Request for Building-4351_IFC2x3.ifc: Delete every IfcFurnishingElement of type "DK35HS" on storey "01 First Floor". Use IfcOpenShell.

First a look at what the model holds.

```python
import ifcopenshell
import ifcopenshell.util.element

model = ifcopenshell.open("Building-4351_IFC2x3.ifc")
print(model.schema)
storey = next(s for s in model.by_type("IfcBuildingStorey") if s.Name == "01 First Floor")
furniture = [e for e in ifcopenshell.util.element.get_decomposition(storey) if e.is_a("IfcFurnishingElement")]
seen = {}
for e in furniture:
    element_type = ifcopenshell.util.element.get_type(e)
    name = element_type.Name if element_type not in (None, e) else None
    seen[name] = seen.get(name, 0) + 1
for name, count in sorted(seen.items(), key=str):
    print(count, "x", name)
```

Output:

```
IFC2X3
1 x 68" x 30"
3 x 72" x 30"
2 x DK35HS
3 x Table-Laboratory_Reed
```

```python
import ifcopenshell
import ifcopenshell.api.root
import ifcopenshell.util.element

model = ifcopenshell.open("Building-4351_IFC2x3.ifc")

storey = next(s for s in model.by_type("IfcBuildingStorey") if s.Name == "01 First Floor")
furniture = [e for e in ifcopenshell.util.element.get_decomposition(storey) if e.is_a("IfcFurnishingElement")]
targets = [e for e in furniture if (t := ifcopenshell.util.element.get_type(e)) not in (None, e) and t.Name == "DK35HS"]

for e in targets:
    ifcopenshell.api.root.remove_product(model, product=e)
print(len(targets), "removed")

model.write("Building-4351_IFC2x3_edited.ifc")
```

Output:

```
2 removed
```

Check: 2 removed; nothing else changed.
